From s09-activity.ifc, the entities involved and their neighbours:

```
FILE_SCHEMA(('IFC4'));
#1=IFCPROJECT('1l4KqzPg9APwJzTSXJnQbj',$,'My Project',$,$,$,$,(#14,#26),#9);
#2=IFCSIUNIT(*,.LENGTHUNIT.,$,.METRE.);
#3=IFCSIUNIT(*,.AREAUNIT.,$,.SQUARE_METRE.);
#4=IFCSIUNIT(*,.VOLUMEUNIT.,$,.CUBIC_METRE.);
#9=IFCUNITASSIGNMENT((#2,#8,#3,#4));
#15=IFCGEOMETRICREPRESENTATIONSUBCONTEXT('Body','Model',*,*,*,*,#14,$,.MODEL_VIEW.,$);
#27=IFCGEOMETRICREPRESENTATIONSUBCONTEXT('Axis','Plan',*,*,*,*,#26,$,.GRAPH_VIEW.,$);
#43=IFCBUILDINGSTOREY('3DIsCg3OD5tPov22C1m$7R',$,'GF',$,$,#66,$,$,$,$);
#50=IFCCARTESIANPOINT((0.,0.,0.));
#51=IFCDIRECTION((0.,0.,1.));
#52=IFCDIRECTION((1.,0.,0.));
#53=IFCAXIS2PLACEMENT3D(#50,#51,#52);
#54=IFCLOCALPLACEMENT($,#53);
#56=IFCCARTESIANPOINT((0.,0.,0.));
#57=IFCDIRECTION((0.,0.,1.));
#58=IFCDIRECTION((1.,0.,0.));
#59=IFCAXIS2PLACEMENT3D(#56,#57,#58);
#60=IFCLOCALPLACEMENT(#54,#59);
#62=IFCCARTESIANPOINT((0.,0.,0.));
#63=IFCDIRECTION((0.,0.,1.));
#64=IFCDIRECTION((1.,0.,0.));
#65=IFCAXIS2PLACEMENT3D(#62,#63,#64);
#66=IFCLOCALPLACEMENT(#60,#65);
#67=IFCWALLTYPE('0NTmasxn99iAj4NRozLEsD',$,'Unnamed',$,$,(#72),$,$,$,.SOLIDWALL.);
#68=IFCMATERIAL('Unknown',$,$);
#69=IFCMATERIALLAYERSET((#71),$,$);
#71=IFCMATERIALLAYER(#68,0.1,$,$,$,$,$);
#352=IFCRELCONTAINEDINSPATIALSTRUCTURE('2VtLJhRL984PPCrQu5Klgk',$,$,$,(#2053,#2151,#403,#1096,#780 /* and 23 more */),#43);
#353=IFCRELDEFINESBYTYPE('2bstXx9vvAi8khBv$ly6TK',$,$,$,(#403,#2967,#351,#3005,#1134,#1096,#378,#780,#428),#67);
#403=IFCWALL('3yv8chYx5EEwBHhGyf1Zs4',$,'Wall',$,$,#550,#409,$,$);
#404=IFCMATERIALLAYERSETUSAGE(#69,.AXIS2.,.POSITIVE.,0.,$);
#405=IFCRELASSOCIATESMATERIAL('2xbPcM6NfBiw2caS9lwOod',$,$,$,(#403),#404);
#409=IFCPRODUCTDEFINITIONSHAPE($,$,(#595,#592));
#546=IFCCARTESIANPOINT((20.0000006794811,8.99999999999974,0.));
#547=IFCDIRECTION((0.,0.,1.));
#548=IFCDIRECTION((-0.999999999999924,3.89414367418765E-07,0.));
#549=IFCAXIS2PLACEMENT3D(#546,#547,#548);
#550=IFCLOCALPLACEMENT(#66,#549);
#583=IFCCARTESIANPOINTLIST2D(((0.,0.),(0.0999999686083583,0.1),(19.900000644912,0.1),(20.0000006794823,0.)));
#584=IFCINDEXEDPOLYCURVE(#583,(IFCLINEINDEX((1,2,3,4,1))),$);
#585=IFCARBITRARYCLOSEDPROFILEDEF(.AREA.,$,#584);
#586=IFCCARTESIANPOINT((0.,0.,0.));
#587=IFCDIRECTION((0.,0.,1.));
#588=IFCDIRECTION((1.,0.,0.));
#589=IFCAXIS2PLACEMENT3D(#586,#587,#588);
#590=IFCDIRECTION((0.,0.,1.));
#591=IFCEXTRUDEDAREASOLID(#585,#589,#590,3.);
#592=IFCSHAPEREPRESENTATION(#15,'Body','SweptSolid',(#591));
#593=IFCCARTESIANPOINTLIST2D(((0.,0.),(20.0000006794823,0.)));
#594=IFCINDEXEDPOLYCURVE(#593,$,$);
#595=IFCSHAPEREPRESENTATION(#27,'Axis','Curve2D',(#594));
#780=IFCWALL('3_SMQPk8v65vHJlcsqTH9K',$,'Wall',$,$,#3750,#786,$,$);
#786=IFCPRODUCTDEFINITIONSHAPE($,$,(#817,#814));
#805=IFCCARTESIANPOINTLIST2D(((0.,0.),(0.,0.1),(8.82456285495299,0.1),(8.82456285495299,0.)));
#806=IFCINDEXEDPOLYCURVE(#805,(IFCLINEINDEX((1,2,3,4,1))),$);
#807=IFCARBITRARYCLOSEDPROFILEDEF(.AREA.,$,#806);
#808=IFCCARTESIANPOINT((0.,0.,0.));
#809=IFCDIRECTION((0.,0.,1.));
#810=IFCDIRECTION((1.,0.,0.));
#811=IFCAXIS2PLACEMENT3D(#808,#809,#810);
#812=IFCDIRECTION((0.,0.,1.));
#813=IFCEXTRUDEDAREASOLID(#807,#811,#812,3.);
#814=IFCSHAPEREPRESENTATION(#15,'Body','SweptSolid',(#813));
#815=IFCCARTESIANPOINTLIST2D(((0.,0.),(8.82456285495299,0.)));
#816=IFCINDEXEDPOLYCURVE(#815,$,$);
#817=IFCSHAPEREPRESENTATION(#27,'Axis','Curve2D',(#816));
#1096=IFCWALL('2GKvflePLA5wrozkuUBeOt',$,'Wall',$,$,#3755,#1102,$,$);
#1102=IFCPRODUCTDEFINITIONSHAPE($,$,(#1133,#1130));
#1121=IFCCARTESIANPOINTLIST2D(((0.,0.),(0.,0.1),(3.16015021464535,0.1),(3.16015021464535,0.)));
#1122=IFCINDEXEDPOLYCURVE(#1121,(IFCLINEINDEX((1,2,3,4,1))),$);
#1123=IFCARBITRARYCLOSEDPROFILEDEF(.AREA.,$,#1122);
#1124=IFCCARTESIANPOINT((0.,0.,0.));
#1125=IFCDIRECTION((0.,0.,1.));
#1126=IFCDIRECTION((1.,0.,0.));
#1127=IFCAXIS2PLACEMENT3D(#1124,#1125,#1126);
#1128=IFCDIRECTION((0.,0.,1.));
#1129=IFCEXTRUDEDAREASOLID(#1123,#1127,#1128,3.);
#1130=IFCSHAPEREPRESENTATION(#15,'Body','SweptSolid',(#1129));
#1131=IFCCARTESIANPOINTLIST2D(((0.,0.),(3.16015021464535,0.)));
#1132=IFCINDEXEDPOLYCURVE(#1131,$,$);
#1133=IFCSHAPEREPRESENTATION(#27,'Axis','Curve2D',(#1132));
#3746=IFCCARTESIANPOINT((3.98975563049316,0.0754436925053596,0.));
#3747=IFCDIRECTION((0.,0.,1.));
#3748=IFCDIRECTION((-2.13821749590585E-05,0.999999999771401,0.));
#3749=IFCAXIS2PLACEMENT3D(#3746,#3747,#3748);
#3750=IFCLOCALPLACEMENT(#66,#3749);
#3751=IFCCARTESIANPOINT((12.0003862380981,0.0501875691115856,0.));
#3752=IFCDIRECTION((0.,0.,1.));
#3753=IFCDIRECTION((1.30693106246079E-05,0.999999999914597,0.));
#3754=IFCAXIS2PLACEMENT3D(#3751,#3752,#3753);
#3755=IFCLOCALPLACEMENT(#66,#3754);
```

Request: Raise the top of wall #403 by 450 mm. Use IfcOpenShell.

```python
import ifcopenshell
import ifcopenshell.geom
import ifcopenshell.util.representation
import ifcopenshell.util.shape

model = ifcopenshell.open("s09-activity.ifc")
settings = ifcopenshell.geom.settings()


def volume(element):
    """Net volume in cubic metres, openings subtracted."""
    shape = ifcopenshell.geom.create_shape(settings, element)
    return ifcopenshell.util.shape.get_volume(shape.geometry)


wall = model.by_guid("3yv8chYx5EEwBHhGyf1Zs4")
before = volume(wall)

body = ifcopenshell.util.representation.get_representation(wall, "Model", "Body")
solid = body.Items[0]
old_height = solid.Depth
solid.Depth += 0.45
after = volume(wall)

print(f"height {old_height:g} -> {solid.Depth:g}, volume {before:.3f} -> {after:.3f} m3")

model.write("s09-activity_rev.ifc")
```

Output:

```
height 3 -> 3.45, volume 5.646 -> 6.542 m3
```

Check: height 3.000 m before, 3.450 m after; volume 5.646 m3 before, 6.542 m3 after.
